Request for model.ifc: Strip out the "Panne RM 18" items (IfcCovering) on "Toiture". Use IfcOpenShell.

First a look at what the model holds.

```python
import ifcopenshell
import ifcopenshell.util.element

model = ifcopenshell.open("model.ifc")
print(model.schema)
storey = next(s for s in model.by_type("IfcBuildingStorey") if s.Name == "Toiture")
coverings = [e for e in ifcopenshell.util.element.get_decomposition(storey) if e.is_a("IfcCovering")]
seen = {}
for e in coverings:
    element_type = ifcopenshell.util.element.get_type(e)
    name = element_type.Name if element_type not in (None, e) else None
    seen[name] = seen.get(name, 0) + 1
for name, count in sorted(seen.items(), key=str):
    print(count, "x", name)
```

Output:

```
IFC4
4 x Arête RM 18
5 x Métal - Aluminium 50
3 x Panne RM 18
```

```python
import ifcopenshell
import ifcopenshell.api.root
import ifcopenshell.util.element

model = ifcopenshell.open("model.ifc")

storey = next(s for s in model.by_type("IfcBuildingStorey") if s.Name == "Toiture")
coverings = [e for e in ifcopenshell.util.element.get_decomposition(storey) if e.is_a("IfcCovering")]
targets = [e for e in coverings if (t := ifcopenshell.util.element.get_type(e)) not in (None, e) and t.Name == "Panne RM 18"]

for e in targets:
    ifcopenshell.api.root.remove_product(model, product=e)
print(len(targets), "removed")

model.write("model-out.ifc")
```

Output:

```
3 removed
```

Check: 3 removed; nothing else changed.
